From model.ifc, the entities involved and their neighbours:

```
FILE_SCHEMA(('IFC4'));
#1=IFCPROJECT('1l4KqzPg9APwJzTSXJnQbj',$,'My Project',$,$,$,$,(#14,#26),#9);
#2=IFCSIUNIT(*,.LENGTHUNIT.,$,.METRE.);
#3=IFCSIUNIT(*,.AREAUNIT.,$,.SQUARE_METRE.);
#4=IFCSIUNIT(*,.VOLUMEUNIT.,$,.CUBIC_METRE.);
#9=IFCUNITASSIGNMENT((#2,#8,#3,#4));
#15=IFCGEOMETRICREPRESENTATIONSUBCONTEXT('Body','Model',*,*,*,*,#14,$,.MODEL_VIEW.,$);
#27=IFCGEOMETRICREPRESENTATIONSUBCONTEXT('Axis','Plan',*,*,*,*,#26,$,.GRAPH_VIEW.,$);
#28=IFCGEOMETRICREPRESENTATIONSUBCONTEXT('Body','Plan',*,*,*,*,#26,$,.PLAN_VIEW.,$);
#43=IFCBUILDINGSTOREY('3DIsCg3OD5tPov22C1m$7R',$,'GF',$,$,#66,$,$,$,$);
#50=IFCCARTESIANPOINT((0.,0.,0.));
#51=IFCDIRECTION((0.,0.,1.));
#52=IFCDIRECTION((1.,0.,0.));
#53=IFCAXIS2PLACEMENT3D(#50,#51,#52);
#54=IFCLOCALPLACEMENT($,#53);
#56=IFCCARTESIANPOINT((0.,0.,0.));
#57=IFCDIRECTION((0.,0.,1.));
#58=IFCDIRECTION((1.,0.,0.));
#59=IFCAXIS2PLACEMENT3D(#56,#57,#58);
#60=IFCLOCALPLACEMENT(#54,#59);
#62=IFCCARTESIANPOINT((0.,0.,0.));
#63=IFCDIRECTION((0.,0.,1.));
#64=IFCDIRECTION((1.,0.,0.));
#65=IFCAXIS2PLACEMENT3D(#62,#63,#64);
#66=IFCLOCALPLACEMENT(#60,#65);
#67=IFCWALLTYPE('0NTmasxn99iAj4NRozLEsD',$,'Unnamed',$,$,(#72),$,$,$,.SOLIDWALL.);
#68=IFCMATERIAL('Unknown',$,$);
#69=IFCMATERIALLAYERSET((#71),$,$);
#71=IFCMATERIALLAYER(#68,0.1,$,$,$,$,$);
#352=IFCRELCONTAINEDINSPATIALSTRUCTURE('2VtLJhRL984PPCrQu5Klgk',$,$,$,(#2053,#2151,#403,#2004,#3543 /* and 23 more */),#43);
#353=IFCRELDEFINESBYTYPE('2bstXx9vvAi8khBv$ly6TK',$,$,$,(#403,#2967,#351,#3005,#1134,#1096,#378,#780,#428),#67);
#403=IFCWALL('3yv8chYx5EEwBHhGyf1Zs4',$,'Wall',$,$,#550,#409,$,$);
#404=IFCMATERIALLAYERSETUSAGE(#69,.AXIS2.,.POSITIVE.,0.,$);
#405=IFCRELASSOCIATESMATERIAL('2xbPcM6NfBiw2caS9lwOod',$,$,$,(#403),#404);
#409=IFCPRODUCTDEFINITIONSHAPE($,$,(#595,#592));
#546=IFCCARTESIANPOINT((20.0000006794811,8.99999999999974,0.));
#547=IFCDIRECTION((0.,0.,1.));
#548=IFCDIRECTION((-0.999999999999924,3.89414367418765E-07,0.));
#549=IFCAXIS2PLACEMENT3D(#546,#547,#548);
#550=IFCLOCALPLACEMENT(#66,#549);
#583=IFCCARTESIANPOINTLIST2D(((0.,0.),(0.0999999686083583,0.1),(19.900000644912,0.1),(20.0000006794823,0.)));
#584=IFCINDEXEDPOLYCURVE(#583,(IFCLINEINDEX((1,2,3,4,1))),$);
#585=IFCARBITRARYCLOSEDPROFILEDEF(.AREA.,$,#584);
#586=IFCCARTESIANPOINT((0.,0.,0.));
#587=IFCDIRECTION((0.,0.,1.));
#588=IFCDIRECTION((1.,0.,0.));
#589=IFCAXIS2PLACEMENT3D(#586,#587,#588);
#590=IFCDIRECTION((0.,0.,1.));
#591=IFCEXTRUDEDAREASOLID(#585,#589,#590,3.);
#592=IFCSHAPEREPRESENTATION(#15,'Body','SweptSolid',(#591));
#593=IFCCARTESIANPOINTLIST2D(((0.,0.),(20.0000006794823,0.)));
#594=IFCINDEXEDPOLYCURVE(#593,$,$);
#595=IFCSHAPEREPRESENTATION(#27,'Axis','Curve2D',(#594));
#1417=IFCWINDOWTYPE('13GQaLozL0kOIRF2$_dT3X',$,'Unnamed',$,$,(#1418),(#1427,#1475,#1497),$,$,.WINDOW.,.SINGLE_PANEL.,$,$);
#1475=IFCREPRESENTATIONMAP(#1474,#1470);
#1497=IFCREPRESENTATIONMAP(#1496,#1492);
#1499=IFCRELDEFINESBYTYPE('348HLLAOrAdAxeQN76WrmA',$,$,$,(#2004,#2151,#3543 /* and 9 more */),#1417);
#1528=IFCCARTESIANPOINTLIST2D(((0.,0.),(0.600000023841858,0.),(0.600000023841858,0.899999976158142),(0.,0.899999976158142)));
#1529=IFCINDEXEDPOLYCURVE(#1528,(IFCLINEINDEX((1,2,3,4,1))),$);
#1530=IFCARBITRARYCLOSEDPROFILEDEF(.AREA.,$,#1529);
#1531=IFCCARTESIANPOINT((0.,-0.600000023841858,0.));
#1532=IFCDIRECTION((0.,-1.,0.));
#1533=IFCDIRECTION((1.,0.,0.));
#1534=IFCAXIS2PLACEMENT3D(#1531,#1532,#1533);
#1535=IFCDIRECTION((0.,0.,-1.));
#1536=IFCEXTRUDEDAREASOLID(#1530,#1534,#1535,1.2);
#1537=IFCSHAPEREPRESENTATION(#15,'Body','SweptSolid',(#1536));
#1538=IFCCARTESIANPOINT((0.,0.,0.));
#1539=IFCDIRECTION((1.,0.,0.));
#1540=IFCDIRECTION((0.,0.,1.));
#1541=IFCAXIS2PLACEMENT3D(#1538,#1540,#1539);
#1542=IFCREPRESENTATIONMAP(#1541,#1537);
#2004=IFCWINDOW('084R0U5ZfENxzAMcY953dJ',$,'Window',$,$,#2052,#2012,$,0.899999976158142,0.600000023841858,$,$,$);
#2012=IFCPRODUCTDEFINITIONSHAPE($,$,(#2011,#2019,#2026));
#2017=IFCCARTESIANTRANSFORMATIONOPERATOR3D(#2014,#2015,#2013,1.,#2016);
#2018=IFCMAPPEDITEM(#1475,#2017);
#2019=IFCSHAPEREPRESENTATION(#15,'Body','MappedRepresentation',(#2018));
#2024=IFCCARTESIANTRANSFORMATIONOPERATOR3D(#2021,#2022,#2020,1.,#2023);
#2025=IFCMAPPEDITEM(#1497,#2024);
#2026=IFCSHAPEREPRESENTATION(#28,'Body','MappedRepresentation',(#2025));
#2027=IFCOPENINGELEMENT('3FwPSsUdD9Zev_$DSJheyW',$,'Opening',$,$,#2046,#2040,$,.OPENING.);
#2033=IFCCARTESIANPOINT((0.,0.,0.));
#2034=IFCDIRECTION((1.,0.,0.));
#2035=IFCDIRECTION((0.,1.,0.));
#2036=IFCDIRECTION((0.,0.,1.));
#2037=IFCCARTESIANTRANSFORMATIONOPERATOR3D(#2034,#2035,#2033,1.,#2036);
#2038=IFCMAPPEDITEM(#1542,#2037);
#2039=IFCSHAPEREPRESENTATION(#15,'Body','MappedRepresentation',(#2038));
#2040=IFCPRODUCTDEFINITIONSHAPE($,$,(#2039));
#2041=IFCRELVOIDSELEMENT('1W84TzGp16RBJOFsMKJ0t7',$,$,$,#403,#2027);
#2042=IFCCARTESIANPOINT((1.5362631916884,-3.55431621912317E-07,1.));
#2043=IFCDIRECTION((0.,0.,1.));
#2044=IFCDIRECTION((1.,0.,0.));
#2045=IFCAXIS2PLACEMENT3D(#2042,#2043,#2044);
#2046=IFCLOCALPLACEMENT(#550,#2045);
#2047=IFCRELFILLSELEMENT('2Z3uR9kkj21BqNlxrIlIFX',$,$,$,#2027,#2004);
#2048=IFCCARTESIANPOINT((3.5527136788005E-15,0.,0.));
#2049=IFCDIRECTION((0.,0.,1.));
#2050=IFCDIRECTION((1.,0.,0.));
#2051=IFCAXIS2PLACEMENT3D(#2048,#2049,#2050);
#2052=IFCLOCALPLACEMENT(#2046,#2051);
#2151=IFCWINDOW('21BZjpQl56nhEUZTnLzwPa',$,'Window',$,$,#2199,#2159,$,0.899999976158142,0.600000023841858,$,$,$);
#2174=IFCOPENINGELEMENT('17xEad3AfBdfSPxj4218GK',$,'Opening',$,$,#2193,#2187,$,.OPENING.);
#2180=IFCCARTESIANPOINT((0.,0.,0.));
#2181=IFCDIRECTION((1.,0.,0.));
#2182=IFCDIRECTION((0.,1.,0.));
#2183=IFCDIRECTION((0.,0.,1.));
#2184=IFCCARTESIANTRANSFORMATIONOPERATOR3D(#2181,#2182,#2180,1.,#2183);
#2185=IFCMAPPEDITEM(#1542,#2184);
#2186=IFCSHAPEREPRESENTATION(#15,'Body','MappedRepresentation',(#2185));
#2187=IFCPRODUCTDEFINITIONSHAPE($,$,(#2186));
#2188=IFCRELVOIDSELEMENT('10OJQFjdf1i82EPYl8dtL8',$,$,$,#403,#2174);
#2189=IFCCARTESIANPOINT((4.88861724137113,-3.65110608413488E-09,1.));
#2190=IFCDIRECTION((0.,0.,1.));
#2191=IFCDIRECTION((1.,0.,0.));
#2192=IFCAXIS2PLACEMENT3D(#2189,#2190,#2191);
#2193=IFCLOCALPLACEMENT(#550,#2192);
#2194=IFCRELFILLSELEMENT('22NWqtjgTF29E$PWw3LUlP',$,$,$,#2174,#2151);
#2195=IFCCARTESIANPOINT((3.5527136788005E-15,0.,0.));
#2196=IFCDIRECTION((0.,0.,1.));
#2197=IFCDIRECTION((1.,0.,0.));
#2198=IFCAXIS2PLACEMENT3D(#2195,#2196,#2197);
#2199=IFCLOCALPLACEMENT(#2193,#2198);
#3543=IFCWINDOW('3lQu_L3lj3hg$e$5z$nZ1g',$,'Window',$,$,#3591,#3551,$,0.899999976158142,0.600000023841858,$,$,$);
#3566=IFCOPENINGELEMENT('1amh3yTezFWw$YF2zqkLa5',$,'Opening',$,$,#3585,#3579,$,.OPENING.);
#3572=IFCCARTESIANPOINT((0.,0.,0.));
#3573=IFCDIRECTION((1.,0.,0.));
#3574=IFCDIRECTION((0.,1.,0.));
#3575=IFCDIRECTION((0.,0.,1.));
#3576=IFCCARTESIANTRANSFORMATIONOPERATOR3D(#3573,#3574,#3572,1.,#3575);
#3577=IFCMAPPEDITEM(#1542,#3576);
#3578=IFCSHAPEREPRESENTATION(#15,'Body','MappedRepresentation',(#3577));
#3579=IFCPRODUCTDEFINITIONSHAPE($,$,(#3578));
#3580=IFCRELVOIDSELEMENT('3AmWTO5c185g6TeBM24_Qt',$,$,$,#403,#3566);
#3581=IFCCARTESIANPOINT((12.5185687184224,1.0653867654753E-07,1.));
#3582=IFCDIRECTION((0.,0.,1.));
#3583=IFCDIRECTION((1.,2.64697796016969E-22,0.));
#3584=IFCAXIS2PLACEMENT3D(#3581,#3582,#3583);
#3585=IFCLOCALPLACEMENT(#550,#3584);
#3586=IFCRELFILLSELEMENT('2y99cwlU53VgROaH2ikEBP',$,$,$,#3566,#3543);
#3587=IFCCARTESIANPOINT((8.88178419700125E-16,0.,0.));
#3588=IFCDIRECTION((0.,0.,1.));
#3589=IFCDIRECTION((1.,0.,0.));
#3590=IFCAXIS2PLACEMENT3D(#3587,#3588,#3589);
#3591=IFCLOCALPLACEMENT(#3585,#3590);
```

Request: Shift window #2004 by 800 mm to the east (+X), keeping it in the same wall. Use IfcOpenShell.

```python
import ifcopenshell
import ifcopenshell.api.geometry
import ifcopenshell.util.placement
import ifcopenshell.util.unit

model = ifcopenshell.open("model.ifc")
unit_scale = ifcopenshell.util.unit.calculate_unit_scale(model)

window = model.by_id(2004)
opening = window.FillsVoids[0].RelatingOpeningElement
wall = opening.VoidsElements[0].RelatingBuildingElement

wall_matrix = ifcopenshell.util.placement.get_local_placement(wall.ObjectPlacement)
shift = wall_matrix[:3, 0] * -0.8 / unit_scale
before = ifcopenshell.util.placement.get_local_placement(window.ObjectPlacement)[:3, 3].copy()

# The window is placed relative to its opening, so it follows when the opening moves.
matrix = ifcopenshell.util.placement.get_local_placement(opening.ObjectPlacement)
matrix[:3, 3] += shift
ifcopenshell.api.geometry.edit_object_placement(
    model, product=opening, matrix=matrix, is_si=False, should_transform_children=True
)

after = ifcopenshell.util.placement.get_local_placement(window.ObjectPlacement)[:3, 3]
print("window moved by", (after - before).round(3) + 0.0)

model.write("model-out.ifc")
```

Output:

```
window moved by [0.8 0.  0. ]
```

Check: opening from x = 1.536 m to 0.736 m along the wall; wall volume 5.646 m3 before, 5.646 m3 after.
